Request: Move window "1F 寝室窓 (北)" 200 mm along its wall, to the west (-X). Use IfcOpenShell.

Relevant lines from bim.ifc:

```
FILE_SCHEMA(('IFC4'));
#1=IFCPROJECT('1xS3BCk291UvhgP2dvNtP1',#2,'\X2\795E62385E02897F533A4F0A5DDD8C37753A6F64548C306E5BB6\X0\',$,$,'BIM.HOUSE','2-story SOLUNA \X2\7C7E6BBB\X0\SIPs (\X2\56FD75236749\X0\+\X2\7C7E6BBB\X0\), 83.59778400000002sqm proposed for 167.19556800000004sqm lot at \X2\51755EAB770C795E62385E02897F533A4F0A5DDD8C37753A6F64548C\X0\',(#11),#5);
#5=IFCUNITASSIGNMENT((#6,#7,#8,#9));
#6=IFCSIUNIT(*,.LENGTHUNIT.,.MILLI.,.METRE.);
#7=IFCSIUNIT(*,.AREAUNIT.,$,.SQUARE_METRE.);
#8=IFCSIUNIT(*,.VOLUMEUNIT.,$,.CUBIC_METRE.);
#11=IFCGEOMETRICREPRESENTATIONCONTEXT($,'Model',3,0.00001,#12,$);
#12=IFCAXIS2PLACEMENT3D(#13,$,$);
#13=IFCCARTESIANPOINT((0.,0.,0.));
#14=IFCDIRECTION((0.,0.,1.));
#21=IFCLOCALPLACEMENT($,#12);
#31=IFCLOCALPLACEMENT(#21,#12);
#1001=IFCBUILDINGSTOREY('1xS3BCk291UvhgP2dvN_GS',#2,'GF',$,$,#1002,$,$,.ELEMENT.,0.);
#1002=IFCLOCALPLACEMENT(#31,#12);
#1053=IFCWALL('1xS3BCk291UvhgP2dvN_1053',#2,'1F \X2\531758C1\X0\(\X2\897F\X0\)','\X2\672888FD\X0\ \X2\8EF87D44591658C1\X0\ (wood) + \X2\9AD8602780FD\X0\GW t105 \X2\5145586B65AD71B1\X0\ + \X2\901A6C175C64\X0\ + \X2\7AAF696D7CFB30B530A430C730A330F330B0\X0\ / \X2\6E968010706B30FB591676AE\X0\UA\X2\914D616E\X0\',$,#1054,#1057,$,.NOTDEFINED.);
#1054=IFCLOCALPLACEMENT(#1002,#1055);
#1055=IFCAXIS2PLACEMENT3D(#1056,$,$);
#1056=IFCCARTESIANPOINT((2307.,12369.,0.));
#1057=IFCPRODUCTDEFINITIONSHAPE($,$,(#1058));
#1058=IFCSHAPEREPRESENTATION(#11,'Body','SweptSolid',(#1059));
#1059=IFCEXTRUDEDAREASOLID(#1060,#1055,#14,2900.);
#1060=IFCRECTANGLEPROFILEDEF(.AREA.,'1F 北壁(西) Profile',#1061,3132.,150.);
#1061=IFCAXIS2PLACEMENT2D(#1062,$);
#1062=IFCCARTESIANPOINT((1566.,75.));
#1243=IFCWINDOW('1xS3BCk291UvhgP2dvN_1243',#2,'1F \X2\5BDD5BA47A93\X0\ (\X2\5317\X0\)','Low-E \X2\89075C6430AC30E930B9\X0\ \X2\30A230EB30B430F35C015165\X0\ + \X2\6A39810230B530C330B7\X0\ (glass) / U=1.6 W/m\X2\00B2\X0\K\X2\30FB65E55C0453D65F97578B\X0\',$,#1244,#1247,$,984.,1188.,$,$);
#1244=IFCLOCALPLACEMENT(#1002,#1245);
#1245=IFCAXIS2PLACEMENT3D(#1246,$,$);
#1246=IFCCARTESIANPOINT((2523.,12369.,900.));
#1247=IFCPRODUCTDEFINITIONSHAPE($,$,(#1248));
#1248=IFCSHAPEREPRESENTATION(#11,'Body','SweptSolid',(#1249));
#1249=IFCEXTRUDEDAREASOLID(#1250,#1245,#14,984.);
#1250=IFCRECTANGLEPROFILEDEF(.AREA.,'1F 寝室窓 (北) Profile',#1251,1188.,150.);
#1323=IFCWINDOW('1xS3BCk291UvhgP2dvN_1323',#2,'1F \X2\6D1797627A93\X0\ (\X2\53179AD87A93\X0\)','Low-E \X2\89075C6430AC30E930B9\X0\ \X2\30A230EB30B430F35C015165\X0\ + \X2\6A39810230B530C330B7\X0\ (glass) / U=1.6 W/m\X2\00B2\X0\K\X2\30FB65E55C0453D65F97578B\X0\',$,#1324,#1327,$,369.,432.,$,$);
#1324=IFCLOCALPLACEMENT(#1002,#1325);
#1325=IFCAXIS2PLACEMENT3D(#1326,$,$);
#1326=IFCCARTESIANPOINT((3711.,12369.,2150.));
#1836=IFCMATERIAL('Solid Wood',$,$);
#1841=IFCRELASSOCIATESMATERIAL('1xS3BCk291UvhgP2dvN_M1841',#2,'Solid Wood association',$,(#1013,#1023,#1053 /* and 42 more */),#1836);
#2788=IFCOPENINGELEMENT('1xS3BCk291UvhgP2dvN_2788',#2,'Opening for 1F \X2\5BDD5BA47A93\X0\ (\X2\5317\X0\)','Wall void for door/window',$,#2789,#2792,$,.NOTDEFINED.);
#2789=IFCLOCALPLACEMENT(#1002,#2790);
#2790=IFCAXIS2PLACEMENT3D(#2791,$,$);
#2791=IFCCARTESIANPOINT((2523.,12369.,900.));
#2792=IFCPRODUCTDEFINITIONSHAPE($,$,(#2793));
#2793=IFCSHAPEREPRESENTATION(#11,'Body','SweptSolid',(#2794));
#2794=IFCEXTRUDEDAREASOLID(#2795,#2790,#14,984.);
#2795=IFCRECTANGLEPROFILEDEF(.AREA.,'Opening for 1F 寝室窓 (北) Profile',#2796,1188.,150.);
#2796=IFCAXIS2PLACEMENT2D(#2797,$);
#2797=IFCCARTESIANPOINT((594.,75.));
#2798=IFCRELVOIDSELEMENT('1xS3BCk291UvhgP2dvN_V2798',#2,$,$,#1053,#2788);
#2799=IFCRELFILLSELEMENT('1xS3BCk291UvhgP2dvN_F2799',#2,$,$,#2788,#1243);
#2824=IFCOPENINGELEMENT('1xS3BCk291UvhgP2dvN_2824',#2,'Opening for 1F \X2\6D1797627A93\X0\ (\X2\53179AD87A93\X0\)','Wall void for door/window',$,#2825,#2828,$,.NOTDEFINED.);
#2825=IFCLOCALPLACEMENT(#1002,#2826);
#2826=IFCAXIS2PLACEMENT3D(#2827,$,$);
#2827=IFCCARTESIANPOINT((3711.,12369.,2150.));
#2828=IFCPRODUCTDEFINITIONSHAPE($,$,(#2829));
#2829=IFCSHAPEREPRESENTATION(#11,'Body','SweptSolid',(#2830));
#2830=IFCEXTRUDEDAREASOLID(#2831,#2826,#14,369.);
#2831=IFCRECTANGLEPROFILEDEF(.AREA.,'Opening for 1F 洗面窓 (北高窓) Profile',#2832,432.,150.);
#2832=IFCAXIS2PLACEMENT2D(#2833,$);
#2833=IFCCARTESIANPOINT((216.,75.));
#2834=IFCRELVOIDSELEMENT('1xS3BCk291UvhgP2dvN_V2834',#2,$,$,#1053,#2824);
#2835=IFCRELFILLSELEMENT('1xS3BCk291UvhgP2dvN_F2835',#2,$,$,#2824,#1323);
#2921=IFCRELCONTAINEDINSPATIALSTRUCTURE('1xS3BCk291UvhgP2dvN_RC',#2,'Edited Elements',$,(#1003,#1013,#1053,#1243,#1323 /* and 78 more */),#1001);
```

```python
import ifcopenshell
import ifcopenshell.api.geometry
import ifcopenshell.util.placement
import ifcopenshell.util.unit

model = ifcopenshell.open("bim.ifc")
unit_scale = ifcopenshell.util.unit.calculate_unit_scale(model)

window = model.by_guid("1xS3BCk291UvhgP2dvN_1243")
opening = window.FillsVoids[0].RelatingOpeningElement
wall = opening.VoidsElements[0].RelatingBuildingElement

wall_matrix = ifcopenshell.util.placement.get_local_placement(wall.ObjectPlacement)
shift = wall_matrix[:3, 0] * -0.2 / unit_scale
before = ifcopenshell.util.placement.get_local_placement(window.ObjectPlacement)[:3, 3].copy()

# The window is not placed relative to its opening, so move both.
for product in (opening, window):
    matrix = ifcopenshell.util.placement.get_local_placement(product.ObjectPlacement)
    matrix[:3, 3] += shift
    ifcopenshell.api.geometry.edit_object_placement(model, product=product, matrix=matrix, is_si=False)

after = ifcopenshell.util.placement.get_local_placement(window.ObjectPlacement)[:3, 3]
print("window moved by", (after - before).round(3) + 0.0)

model.write("bim_v2.ifc")
```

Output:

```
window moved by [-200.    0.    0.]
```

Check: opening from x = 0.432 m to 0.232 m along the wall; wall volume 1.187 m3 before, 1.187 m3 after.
